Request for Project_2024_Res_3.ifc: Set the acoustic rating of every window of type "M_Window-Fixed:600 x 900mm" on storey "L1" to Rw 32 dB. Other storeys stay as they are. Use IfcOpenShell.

First a look at what the model holds.

```python
import ifcopenshell
import ifcopenshell.util.element

model = ifcopenshell.open("Project_2024_Res_3.ifc")
print(model.schema)
storey = next(s for s in model.by_type("IfcBuildingStorey") if s.Name == "L1")
windows = [e for e in ifcopenshell.util.element.get_decomposition(storey) if e.is_a("IfcWindow")]
seen = {}
for e in windows:
    element_type = ifcopenshell.util.element.get_type(e)
    key = (element_type.Name if element_type != e and element_type else None, ifcopenshell.util.element.get_pset(e, "Pset_WindowCommon", "AcousticRating"))
    seen[key] = seen.get(key, 0) + 1
for (name, value), count in sorted(seen.items(), key=str):
    print(count, "x", name, "|", value)
```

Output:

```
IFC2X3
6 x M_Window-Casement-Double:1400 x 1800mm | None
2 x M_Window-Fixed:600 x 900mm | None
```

```python
import ifcopenshell
import ifcopenshell.api.pset
import ifcopenshell.util.element

model = ifcopenshell.open("Project_2024_Res_3.ifc")

storey = next(s for s in model.by_type("IfcBuildingStorey") if s.Name == "L1")
windows = [e for e in ifcopenshell.util.element.get_decomposition(storey) if e.is_a("IfcWindow")]

count = 0
for e in windows:
    element_type = ifcopenshell.util.element.get_type(e)
    if element_type in (None, e) or element_type.Name != "M_Window-Fixed:600 x 900mm":
        continue
    # add_pset returns the element's existing set when there is one.
    pset = ifcopenshell.api.pset.add_pset(model, product=e, name="Pset_WindowCommon")
    ifcopenshell.api.pset.edit_pset(model, pset=pset, properties={"AcousticRating": "Rw 32 dB"})
    count += 1

print(count, "windows updated")

model.write("Project_2024_Res_3_v2.ifc")
```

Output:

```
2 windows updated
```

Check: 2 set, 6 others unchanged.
